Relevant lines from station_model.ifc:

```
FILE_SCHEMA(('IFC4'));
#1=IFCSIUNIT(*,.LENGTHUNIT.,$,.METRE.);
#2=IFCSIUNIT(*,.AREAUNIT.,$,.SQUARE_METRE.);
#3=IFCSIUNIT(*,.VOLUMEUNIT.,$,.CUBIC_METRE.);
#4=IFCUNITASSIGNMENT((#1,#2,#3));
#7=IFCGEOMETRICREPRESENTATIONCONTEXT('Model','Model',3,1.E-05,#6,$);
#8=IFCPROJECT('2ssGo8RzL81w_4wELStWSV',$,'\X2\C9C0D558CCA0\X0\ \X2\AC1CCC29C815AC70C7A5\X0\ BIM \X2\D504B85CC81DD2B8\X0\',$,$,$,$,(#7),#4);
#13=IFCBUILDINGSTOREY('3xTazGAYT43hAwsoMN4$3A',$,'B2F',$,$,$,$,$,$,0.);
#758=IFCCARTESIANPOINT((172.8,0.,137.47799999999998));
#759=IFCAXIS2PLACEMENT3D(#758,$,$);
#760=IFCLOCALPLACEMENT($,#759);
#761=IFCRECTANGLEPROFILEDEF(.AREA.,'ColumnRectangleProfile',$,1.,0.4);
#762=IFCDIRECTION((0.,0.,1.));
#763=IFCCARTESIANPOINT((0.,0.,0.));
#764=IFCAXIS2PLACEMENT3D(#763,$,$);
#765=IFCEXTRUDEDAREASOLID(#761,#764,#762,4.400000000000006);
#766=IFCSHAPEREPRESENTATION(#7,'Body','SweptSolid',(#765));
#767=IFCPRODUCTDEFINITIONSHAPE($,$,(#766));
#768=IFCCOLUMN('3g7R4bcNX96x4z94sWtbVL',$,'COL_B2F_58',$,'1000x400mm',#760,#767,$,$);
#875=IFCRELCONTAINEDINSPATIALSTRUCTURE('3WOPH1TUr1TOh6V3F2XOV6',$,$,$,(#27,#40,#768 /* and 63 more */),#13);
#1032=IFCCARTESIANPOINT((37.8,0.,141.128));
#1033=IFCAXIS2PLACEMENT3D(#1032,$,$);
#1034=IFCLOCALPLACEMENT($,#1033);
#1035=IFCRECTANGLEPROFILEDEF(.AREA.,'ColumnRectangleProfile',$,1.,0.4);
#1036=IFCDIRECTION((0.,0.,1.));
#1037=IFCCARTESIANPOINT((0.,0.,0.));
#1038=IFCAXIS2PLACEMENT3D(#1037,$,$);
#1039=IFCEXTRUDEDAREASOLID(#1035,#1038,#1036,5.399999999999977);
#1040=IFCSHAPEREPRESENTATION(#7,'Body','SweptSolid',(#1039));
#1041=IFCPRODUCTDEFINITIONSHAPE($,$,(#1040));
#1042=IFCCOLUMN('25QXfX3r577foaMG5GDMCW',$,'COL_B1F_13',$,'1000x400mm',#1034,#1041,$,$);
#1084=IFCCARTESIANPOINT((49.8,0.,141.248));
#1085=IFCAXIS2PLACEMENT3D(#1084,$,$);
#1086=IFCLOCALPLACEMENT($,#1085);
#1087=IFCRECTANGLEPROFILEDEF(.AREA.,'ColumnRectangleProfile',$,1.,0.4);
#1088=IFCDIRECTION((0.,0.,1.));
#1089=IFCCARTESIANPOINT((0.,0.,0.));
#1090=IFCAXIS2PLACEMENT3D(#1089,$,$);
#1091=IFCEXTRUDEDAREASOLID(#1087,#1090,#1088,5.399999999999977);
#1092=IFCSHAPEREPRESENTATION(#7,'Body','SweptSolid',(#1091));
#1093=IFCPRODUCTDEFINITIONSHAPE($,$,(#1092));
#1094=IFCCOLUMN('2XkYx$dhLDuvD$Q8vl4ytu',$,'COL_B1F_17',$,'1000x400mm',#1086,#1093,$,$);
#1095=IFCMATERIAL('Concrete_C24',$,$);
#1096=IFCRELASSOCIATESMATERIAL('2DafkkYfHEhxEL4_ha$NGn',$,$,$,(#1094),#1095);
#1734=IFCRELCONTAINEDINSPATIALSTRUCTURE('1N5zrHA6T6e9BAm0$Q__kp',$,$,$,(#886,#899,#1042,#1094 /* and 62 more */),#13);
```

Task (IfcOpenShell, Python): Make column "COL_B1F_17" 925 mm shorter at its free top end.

```python
import ifcopenshell
import ifcopenshell.util.unit

model = ifcopenshell.open("station_model.ifc")
unit_scale = ifcopenshell.util.unit.calculate_unit_scale(model)

member = model.by_id(1094)
change = -0.925 / unit_scale

# The extrusion runs towards the end named, so only its depth changes.
body = next(r for r in member.Representation.Representations if r.RepresentationIdentifier == "Body")
solid = body.Items[0]
old_length = solid.Depth
solid.Depth += change

print(f"length {old_length:g} -> {solid.Depth:g}")

model.write("station_model_edited.ifc")
```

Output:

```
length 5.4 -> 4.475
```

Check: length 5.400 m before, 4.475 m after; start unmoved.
